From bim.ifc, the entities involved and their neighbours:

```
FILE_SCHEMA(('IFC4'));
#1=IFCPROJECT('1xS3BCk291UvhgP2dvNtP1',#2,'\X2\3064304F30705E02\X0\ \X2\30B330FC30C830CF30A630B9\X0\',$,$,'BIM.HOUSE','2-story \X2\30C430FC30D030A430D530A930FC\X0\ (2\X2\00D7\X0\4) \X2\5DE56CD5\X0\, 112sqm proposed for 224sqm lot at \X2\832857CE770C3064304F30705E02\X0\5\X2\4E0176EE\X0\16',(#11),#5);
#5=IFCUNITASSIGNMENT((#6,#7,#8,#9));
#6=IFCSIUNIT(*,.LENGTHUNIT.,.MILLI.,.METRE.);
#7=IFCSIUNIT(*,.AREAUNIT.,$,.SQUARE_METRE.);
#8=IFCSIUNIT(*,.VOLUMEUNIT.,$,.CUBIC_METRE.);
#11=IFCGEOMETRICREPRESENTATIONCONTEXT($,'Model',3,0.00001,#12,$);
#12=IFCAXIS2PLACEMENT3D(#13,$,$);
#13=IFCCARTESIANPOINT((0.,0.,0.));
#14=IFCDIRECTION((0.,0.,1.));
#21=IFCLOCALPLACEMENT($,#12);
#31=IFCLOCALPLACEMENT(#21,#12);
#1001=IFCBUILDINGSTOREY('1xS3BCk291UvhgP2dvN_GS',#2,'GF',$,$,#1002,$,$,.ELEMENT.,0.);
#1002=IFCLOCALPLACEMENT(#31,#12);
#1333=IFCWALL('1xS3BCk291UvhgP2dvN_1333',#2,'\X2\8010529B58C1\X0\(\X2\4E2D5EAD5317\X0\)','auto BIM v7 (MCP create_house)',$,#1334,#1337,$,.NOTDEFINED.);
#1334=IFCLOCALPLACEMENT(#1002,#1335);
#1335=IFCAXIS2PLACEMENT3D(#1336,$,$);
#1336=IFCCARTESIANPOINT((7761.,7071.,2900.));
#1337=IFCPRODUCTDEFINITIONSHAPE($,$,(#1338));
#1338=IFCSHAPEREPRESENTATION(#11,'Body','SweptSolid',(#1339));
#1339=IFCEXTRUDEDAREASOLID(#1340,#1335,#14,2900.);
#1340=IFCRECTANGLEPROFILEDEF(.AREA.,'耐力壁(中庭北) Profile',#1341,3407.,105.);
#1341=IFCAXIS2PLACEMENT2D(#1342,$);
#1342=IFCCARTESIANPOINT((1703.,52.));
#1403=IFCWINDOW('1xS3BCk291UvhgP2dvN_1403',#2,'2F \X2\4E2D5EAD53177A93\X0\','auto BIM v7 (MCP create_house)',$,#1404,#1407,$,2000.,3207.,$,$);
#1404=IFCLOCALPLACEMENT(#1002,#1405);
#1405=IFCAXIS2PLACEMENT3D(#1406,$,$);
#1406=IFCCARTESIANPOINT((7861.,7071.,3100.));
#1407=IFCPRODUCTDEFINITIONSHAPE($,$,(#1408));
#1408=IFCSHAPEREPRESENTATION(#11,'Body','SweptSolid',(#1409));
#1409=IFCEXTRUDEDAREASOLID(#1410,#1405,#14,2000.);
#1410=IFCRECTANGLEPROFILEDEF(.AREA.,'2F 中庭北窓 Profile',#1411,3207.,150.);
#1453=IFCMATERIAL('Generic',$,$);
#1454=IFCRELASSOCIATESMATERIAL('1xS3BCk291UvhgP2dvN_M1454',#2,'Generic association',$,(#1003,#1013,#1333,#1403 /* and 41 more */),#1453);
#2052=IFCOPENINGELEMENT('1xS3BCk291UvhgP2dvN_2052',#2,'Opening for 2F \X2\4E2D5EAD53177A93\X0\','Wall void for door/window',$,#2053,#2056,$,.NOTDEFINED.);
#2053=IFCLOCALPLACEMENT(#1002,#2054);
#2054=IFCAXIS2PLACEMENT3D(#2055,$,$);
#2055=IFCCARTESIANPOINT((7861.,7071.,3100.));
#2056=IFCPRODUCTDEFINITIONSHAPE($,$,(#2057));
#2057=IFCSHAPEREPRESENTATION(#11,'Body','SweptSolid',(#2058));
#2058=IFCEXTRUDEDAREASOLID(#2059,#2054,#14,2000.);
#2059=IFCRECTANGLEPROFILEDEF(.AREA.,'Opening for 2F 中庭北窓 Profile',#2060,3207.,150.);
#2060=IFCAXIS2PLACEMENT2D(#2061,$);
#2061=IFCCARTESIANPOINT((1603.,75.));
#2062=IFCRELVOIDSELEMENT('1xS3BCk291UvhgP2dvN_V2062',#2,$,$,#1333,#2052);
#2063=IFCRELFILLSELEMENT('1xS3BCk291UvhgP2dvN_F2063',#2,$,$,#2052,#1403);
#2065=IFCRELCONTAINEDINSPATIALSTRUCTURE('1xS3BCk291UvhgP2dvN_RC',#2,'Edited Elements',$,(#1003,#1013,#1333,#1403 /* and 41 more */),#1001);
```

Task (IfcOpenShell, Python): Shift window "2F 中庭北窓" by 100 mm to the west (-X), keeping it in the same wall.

```python
import ifcopenshell
import ifcopenshell.api.geometry
import ifcopenshell.util.placement

model = ifcopenshell.open("bim.ifc")

window = model.by_guid("1xS3BCk291UvhgP2dvN_1403")
opening = window.FillsVoids[0].RelatingOpeningElement
wall = opening.VoidsElements[0].RelatingBuildingElement

wall_matrix = ifcopenshell.util.placement.get_local_placement(wall.ObjectPlacement)
shift = wall_matrix[:3, 0] * -100.0
before = ifcopenshell.util.placement.get_local_placement(window.ObjectPlacement)[:3, 3].copy()

# The window is not placed relative to its opening, so move both.
for product in (opening, window):
    matrix = ifcopenshell.util.placement.get_local_placement(product.ObjectPlacement)
    matrix[:3, 3] += shift
    ifcopenshell.api.geometry.edit_object_placement(model, product=product, matrix=matrix, is_si=False)

after = ifcopenshell.util.placement.get_local_placement(window.ObjectPlacement)[:3, 3]
print("window moved by", (after - before).round(3) + 0.0)

model.write("bim-out.ifc")
```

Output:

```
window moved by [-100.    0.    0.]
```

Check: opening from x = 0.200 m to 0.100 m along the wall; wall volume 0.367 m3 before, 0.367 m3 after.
